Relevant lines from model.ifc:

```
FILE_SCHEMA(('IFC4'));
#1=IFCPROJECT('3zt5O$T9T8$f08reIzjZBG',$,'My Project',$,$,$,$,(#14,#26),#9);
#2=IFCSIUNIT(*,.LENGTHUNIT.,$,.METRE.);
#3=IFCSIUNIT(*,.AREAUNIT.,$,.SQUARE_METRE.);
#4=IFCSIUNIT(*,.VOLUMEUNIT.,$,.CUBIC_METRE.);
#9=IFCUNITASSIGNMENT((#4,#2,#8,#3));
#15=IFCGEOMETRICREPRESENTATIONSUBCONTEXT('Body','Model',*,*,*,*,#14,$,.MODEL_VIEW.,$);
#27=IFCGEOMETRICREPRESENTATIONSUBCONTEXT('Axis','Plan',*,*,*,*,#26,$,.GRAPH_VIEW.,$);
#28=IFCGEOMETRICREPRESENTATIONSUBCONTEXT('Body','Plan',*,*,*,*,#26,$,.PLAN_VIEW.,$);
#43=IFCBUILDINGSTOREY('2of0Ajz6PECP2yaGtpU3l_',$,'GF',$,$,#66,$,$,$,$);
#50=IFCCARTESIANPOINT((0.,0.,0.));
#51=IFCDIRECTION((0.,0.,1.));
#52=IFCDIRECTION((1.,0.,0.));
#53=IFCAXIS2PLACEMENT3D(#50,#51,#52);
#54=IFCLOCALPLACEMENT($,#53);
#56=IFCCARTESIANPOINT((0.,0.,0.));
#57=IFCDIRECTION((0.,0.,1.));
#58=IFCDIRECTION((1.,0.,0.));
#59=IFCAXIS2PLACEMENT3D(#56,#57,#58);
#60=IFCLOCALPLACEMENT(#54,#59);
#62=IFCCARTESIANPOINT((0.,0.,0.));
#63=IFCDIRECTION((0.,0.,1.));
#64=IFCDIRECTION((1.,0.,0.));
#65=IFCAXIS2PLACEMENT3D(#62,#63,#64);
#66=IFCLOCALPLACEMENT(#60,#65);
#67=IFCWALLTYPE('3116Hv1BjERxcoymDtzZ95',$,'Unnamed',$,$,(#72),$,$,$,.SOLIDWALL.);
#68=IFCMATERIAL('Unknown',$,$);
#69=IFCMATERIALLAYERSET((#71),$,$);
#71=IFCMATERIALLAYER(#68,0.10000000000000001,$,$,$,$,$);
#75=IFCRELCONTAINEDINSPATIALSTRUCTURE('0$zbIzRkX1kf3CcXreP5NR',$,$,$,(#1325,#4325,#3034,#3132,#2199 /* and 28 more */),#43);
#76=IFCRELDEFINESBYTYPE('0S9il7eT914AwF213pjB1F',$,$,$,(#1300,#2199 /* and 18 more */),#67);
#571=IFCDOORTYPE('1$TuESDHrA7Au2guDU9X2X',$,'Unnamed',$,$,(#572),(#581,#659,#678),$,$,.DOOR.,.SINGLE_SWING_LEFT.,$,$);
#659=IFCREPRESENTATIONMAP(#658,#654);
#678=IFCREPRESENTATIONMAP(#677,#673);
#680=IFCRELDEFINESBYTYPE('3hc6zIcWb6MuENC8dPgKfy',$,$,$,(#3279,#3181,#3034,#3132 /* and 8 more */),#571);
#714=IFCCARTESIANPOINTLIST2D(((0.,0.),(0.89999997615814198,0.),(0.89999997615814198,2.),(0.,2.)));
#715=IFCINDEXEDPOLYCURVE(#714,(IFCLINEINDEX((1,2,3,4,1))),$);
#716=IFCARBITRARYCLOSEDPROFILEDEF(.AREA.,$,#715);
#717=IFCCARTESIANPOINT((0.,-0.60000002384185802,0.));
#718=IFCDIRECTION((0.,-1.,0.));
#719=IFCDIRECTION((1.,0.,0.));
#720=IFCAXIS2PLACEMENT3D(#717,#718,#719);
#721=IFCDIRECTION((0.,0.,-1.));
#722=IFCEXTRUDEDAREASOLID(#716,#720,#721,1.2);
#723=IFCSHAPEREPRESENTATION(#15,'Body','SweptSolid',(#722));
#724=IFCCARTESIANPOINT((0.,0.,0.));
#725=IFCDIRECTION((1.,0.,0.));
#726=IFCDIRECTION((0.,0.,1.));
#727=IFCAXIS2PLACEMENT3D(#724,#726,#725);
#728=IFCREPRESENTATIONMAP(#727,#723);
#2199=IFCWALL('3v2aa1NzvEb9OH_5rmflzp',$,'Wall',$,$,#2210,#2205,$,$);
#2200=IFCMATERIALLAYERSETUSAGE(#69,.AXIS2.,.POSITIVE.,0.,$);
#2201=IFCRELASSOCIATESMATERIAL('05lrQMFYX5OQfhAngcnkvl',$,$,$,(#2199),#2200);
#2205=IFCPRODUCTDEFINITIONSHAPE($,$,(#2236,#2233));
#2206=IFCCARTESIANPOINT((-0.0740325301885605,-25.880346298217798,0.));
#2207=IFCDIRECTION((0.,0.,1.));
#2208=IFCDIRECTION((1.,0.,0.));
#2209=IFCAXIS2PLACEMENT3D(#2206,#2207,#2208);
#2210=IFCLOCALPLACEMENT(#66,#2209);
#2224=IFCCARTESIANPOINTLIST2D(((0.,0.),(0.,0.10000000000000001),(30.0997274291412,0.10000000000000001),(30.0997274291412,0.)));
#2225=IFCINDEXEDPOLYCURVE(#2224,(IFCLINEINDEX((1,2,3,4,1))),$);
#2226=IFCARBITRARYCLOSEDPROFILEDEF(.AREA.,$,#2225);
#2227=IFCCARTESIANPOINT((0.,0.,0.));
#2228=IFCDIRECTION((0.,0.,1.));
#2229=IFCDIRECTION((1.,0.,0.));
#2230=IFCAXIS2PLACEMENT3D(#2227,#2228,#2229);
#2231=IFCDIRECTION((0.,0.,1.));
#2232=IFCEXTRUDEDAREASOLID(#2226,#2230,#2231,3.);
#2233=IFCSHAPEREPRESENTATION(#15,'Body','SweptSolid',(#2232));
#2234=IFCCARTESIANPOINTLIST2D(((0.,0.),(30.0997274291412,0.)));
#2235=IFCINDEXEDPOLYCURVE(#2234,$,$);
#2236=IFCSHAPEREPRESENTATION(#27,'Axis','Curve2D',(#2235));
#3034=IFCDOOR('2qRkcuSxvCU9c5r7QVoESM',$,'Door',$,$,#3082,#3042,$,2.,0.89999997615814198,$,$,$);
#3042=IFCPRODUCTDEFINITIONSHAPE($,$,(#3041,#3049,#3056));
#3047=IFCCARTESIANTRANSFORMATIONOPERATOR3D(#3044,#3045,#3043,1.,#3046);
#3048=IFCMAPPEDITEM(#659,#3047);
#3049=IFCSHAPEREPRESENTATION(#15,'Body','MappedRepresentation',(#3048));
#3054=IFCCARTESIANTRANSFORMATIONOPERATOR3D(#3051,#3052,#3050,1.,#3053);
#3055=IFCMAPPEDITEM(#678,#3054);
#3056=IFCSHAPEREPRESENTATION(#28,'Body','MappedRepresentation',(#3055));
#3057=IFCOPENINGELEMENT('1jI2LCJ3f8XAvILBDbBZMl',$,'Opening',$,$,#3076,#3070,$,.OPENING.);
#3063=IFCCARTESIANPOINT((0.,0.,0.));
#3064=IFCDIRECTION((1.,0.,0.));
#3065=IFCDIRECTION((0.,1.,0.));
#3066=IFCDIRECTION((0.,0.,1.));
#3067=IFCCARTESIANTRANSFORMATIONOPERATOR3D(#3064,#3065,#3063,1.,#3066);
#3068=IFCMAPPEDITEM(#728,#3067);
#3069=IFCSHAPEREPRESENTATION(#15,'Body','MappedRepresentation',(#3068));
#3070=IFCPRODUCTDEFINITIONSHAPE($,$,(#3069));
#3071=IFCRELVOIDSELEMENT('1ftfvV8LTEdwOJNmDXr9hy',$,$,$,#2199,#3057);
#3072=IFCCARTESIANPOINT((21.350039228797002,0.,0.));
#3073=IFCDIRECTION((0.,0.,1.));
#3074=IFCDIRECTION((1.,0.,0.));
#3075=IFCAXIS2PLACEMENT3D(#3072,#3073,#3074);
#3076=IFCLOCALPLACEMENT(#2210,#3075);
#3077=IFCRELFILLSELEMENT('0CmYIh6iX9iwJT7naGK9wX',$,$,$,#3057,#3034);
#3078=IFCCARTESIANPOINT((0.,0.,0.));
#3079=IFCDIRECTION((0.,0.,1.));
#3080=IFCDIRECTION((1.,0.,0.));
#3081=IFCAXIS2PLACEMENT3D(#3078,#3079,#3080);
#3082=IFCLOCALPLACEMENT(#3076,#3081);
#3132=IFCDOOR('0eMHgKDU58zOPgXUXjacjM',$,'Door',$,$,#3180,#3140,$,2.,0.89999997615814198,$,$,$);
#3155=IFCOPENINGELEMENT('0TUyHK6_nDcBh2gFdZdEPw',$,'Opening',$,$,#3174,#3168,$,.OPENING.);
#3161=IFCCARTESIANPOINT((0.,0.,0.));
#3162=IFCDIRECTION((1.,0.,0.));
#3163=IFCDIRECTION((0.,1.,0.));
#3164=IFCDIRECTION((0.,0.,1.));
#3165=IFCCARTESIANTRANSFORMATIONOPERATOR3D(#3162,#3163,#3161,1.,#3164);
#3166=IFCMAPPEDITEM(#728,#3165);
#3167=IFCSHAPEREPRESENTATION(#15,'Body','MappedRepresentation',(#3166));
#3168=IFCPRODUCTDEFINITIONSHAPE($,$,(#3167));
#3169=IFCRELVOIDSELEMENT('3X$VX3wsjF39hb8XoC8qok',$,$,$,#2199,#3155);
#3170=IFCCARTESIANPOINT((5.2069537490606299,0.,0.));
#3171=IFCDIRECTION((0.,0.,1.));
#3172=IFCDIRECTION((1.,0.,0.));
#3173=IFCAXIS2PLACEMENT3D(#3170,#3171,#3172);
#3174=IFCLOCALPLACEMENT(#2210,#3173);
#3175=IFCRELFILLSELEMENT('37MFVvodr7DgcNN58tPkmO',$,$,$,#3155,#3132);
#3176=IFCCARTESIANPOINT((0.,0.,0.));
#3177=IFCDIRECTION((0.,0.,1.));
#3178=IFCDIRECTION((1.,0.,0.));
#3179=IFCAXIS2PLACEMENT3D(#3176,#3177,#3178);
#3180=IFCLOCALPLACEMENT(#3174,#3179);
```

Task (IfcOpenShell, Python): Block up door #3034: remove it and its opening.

```python
import ifcopenshell
import ifcopenshell.api.feature
import ifcopenshell.api.root
import ifcopenshell.geom
import ifcopenshell.util.shape

model = ifcopenshell.open("model.ifc")
settings = ifcopenshell.geom.settings()


def volume(element):
    """Net volume in cubic metres, openings subtracted."""
    shape = ifcopenshell.geom.create_shape(settings, element)
    return ifcopenshell.util.shape.get_volume(shape.geometry)


door = model.by_id(3034)
opening = door.FillsVoids[0].RelatingOpeningElement
wall = opening.VoidsElements[0].RelatingBuildingElement
before = volume(wall)

ifcopenshell.api.root.remove_product(model, product=door)
ifcopenshell.api.feature.remove_feature(model, feature=opening)

after = volume(wall)

print(f"wall volume {before:.3f} -> {after:.3f} m3")

model.write("model_v2.ifc")
```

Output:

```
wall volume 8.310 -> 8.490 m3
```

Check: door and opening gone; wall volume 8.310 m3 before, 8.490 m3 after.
